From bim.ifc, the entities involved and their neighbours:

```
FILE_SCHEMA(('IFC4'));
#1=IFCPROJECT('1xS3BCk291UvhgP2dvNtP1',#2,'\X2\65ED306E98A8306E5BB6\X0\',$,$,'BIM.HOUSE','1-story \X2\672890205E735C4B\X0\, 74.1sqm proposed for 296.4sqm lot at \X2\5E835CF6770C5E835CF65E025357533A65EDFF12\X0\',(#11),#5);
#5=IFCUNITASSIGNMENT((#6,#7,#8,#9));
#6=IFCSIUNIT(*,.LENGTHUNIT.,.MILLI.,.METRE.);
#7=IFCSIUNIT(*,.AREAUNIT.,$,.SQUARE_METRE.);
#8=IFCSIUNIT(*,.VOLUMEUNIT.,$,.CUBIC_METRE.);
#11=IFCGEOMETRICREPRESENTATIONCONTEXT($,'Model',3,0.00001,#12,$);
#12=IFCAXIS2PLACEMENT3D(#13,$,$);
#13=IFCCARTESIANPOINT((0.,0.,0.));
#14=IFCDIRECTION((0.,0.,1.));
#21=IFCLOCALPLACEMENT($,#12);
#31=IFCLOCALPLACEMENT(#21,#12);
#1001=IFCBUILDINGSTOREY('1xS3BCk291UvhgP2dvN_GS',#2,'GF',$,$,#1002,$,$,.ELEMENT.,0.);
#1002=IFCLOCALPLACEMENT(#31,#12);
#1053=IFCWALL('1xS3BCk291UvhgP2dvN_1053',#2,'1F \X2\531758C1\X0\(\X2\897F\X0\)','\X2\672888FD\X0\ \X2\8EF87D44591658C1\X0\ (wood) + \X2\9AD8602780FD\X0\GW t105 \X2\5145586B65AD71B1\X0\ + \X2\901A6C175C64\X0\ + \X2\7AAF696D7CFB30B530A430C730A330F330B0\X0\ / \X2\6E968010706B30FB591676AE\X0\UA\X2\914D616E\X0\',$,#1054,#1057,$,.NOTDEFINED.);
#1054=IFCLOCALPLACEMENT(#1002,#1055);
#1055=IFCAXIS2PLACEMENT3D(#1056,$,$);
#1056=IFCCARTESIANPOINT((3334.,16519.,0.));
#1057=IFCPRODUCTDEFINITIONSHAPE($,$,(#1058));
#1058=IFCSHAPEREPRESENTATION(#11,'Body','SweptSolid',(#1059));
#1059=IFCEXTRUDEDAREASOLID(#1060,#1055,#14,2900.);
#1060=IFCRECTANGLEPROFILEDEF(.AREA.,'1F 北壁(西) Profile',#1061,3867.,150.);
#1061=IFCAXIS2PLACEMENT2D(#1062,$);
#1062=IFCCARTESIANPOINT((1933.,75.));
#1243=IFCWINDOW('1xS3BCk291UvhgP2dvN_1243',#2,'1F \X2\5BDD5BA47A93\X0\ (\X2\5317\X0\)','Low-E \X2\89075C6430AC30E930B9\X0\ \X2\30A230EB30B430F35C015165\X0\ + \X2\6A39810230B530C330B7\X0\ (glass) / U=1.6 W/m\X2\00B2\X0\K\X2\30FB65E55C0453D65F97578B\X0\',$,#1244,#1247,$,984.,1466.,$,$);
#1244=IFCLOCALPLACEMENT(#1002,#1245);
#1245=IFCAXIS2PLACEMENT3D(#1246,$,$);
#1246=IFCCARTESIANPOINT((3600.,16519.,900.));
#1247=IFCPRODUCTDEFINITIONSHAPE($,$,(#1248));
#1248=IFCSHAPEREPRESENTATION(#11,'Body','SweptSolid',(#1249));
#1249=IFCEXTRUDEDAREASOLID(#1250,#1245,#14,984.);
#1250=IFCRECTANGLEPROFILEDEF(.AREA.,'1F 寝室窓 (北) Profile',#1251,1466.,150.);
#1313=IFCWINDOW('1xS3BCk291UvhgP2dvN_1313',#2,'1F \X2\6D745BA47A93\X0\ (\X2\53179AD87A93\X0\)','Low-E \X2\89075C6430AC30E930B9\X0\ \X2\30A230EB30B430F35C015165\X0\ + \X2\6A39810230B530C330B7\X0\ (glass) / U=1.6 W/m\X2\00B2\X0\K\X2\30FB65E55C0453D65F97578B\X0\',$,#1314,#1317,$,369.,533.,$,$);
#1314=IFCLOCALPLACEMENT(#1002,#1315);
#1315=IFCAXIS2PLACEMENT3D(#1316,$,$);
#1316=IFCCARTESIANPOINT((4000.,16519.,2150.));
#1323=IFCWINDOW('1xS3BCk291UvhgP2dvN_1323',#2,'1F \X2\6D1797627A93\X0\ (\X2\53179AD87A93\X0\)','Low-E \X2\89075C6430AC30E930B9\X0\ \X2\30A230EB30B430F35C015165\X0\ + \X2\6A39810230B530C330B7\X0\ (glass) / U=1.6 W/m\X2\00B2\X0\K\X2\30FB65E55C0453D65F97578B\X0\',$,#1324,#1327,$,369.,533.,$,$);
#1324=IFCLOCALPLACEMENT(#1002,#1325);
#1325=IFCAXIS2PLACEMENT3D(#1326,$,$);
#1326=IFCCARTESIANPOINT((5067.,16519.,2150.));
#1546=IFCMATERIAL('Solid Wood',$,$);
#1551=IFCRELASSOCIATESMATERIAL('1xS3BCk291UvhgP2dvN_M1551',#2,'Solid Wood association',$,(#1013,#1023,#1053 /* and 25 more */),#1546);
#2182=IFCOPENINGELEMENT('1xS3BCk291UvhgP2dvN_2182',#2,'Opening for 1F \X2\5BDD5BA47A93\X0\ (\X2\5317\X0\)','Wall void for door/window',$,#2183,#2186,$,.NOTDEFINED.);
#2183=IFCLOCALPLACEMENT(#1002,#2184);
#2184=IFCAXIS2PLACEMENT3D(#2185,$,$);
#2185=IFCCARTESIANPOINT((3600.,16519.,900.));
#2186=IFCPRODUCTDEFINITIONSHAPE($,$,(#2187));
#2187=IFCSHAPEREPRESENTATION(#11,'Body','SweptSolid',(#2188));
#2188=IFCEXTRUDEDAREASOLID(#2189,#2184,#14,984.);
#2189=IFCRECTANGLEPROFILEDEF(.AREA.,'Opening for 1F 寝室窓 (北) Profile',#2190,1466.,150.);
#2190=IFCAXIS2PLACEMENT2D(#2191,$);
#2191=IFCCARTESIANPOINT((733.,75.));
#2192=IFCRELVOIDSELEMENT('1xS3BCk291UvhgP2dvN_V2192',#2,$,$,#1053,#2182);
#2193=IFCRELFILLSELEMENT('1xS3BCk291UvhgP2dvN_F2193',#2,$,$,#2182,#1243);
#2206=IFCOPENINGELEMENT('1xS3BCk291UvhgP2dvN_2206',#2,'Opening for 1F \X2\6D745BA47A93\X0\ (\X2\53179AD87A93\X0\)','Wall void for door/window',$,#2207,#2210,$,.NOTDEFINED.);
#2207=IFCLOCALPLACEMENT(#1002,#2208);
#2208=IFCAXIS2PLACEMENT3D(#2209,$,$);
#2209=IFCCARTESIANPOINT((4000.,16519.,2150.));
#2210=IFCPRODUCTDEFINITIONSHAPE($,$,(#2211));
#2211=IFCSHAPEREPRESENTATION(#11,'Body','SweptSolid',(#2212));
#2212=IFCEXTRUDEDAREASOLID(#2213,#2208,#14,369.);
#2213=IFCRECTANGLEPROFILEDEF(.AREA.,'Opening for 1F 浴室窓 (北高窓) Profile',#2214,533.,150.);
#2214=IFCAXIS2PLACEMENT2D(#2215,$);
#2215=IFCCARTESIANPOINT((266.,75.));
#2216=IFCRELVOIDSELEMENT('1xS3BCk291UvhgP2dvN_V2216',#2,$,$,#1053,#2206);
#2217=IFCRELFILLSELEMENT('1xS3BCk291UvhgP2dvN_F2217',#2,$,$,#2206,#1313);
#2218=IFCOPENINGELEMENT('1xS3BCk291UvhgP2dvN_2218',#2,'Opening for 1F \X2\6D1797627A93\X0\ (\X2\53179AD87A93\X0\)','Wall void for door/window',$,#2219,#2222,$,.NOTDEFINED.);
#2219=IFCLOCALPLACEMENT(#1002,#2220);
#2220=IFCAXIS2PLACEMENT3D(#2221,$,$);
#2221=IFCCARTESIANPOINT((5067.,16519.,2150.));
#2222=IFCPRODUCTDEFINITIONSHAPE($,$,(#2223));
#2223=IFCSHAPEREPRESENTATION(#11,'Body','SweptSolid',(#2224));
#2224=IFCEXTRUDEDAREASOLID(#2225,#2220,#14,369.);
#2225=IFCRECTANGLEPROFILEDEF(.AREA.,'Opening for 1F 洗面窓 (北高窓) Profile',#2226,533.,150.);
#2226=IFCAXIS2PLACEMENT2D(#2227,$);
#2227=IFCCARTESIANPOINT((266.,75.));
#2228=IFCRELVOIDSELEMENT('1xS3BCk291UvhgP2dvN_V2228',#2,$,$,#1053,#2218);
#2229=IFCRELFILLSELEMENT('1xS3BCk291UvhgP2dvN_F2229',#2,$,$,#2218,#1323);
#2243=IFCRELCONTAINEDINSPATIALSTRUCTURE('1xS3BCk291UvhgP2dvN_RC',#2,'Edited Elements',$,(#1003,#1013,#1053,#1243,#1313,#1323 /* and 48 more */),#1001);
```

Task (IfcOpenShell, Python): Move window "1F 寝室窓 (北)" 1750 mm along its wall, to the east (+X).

```python
import ifcopenshell
import ifcopenshell.api.geometry
import ifcopenshell.util.placement
import ifcopenshell.util.unit

model = ifcopenshell.open("bim.ifc")
unit_scale = ifcopenshell.util.unit.calculate_unit_scale(model)

window = model.by_guid("1xS3BCk291UvhgP2dvN_1243")
opening = window.FillsVoids[0].RelatingOpeningElement
wall = opening.VoidsElements[0].RelatingBuildingElement

wall_matrix = ifcopenshell.util.placement.get_local_placement(wall.ObjectPlacement)
shift = wall_matrix[:3, 0] * 1.75 / unit_scale
before = ifcopenshell.util.placement.get_local_placement(window.ObjectPlacement)[:3, 3].copy()

# The window is not placed relative to its opening, so move both.
for product in (opening, window):
    matrix = ifcopenshell.util.placement.get_local_placement(product.ObjectPlacement)
    matrix[:3, 3] += shift
    ifcopenshell.api.geometry.edit_object_placement(model, product=product, matrix=matrix, is_si=False)

after = ifcopenshell.util.placement.get_local_placement(window.ObjectPlacement)[:3, 3]
print("window moved by", (after - before).round(3) + 0.0)

model.write("bim_edited.ifc")
```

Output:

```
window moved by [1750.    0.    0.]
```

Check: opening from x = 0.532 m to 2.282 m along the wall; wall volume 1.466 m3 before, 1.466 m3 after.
